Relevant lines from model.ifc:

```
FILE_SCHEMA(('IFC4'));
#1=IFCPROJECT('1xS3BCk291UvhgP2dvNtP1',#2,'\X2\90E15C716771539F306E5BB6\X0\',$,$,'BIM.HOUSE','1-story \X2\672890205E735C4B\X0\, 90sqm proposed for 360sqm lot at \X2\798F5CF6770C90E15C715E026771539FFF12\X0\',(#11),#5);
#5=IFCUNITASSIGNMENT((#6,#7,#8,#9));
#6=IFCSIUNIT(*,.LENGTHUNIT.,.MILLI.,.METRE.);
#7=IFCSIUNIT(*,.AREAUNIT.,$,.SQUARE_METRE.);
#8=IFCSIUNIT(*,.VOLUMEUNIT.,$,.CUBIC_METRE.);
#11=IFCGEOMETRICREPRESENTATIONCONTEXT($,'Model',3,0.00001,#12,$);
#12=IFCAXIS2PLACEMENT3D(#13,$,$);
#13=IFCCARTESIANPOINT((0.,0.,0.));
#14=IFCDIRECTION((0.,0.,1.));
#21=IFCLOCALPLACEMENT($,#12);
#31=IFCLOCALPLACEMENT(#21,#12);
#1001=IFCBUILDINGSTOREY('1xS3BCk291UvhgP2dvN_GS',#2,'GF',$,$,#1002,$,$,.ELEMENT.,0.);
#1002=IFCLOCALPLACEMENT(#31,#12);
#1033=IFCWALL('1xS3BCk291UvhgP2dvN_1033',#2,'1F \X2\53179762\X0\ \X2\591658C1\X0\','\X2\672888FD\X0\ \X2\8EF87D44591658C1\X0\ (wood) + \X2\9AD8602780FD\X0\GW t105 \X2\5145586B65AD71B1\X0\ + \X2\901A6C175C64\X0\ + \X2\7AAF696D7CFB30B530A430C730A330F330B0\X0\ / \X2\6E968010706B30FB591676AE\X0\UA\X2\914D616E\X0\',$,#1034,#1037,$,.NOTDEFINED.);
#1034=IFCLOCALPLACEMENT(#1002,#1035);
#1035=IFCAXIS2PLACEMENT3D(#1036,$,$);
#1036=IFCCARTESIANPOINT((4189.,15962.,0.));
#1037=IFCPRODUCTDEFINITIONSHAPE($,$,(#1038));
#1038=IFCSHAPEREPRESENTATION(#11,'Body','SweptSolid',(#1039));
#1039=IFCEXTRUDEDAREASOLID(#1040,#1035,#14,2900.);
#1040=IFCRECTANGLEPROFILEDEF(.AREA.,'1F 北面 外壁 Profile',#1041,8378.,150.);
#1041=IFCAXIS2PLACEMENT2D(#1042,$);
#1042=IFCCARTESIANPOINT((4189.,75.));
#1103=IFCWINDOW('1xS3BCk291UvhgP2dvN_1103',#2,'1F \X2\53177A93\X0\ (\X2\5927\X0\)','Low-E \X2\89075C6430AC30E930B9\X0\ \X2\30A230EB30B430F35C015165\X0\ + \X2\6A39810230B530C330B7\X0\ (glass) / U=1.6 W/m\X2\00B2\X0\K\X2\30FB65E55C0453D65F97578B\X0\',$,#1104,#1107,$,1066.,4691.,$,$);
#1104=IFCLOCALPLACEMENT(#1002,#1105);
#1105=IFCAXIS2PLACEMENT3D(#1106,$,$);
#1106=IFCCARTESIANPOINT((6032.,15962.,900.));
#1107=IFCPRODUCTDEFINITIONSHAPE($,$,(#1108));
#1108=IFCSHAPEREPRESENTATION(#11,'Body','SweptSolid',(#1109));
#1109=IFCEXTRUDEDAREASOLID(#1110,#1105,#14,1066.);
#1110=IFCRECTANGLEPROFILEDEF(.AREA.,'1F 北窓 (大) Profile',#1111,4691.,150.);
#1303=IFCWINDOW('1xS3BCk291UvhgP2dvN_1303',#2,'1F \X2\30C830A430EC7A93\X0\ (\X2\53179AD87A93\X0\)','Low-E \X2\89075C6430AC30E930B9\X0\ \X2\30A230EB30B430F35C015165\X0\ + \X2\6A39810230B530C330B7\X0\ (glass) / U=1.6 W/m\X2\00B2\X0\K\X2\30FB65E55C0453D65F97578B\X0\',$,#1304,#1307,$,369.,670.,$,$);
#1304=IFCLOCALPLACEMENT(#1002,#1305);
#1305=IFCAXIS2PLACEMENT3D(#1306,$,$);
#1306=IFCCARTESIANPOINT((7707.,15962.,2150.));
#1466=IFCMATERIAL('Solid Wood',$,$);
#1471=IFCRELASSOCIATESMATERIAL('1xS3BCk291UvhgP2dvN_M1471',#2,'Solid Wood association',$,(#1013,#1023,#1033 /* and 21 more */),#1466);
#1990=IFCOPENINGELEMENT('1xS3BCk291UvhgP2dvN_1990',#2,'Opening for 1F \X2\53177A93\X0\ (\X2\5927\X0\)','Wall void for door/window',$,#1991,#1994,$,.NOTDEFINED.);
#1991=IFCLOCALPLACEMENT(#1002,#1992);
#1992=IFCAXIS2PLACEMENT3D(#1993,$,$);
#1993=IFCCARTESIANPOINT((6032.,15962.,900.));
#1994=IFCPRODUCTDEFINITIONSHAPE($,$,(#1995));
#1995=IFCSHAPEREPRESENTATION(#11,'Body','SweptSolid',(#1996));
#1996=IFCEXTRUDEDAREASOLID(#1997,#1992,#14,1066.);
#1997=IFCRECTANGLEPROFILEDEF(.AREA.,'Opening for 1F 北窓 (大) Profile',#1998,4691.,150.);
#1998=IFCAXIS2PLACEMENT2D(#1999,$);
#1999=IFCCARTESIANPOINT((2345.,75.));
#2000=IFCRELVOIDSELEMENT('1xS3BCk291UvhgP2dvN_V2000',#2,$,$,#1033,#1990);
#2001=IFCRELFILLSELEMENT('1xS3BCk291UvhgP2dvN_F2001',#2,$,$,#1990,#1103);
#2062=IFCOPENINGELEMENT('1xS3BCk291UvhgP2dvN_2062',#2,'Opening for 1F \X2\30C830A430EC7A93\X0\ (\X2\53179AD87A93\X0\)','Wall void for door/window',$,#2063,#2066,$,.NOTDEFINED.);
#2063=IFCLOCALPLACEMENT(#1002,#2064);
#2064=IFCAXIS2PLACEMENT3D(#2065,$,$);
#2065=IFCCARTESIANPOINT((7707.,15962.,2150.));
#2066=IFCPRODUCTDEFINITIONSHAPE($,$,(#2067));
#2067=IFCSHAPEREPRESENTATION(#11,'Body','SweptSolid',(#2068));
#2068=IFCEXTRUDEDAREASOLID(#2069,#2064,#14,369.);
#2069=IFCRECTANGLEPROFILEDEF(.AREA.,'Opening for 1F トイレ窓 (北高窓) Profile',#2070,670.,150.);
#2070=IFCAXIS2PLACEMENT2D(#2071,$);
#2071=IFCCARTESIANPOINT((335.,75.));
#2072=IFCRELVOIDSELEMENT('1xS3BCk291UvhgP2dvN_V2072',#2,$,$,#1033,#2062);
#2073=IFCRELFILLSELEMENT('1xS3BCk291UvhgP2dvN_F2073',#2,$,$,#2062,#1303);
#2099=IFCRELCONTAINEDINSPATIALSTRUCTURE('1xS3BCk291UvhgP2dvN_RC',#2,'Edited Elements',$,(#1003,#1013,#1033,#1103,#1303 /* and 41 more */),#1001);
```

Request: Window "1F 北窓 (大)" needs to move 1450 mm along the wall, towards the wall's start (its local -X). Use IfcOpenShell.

```python
import ifcopenshell
import ifcopenshell.api.geometry
import ifcopenshell.util.placement
import ifcopenshell.util.unit

model = ifcopenshell.open("model.ifc")
unit_scale = ifcopenshell.util.unit.calculate_unit_scale(model)

window = model.by_guid("1xS3BCk291UvhgP2dvN_1103")
opening = window.FillsVoids[0].RelatingOpeningElement
wall = opening.VoidsElements[0].RelatingBuildingElement

wall_matrix = ifcopenshell.util.placement.get_local_placement(wall.ObjectPlacement)
shift = wall_matrix[:3, 0] * -1.45 / unit_scale
before = ifcopenshell.util.placement.get_local_placement(window.ObjectPlacement)[:3, 3].copy()

# The window is not placed relative to its opening, so move both.
for product in (opening, window):
    matrix = ifcopenshell.util.placement.get_local_placement(product.ObjectPlacement)
    matrix[:3, 3] += shift
    ifcopenshell.api.geometry.edit_object_placement(model, product=product, matrix=matrix, is_si=False)

after = ifcopenshell.util.placement.get_local_placement(window.ObjectPlacement)[:3, 3]
print("window moved by", (after - before).round(3) + 0.0)

model.write("model_edited.ifc")
```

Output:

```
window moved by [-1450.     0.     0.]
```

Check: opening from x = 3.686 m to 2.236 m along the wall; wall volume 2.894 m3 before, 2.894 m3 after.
